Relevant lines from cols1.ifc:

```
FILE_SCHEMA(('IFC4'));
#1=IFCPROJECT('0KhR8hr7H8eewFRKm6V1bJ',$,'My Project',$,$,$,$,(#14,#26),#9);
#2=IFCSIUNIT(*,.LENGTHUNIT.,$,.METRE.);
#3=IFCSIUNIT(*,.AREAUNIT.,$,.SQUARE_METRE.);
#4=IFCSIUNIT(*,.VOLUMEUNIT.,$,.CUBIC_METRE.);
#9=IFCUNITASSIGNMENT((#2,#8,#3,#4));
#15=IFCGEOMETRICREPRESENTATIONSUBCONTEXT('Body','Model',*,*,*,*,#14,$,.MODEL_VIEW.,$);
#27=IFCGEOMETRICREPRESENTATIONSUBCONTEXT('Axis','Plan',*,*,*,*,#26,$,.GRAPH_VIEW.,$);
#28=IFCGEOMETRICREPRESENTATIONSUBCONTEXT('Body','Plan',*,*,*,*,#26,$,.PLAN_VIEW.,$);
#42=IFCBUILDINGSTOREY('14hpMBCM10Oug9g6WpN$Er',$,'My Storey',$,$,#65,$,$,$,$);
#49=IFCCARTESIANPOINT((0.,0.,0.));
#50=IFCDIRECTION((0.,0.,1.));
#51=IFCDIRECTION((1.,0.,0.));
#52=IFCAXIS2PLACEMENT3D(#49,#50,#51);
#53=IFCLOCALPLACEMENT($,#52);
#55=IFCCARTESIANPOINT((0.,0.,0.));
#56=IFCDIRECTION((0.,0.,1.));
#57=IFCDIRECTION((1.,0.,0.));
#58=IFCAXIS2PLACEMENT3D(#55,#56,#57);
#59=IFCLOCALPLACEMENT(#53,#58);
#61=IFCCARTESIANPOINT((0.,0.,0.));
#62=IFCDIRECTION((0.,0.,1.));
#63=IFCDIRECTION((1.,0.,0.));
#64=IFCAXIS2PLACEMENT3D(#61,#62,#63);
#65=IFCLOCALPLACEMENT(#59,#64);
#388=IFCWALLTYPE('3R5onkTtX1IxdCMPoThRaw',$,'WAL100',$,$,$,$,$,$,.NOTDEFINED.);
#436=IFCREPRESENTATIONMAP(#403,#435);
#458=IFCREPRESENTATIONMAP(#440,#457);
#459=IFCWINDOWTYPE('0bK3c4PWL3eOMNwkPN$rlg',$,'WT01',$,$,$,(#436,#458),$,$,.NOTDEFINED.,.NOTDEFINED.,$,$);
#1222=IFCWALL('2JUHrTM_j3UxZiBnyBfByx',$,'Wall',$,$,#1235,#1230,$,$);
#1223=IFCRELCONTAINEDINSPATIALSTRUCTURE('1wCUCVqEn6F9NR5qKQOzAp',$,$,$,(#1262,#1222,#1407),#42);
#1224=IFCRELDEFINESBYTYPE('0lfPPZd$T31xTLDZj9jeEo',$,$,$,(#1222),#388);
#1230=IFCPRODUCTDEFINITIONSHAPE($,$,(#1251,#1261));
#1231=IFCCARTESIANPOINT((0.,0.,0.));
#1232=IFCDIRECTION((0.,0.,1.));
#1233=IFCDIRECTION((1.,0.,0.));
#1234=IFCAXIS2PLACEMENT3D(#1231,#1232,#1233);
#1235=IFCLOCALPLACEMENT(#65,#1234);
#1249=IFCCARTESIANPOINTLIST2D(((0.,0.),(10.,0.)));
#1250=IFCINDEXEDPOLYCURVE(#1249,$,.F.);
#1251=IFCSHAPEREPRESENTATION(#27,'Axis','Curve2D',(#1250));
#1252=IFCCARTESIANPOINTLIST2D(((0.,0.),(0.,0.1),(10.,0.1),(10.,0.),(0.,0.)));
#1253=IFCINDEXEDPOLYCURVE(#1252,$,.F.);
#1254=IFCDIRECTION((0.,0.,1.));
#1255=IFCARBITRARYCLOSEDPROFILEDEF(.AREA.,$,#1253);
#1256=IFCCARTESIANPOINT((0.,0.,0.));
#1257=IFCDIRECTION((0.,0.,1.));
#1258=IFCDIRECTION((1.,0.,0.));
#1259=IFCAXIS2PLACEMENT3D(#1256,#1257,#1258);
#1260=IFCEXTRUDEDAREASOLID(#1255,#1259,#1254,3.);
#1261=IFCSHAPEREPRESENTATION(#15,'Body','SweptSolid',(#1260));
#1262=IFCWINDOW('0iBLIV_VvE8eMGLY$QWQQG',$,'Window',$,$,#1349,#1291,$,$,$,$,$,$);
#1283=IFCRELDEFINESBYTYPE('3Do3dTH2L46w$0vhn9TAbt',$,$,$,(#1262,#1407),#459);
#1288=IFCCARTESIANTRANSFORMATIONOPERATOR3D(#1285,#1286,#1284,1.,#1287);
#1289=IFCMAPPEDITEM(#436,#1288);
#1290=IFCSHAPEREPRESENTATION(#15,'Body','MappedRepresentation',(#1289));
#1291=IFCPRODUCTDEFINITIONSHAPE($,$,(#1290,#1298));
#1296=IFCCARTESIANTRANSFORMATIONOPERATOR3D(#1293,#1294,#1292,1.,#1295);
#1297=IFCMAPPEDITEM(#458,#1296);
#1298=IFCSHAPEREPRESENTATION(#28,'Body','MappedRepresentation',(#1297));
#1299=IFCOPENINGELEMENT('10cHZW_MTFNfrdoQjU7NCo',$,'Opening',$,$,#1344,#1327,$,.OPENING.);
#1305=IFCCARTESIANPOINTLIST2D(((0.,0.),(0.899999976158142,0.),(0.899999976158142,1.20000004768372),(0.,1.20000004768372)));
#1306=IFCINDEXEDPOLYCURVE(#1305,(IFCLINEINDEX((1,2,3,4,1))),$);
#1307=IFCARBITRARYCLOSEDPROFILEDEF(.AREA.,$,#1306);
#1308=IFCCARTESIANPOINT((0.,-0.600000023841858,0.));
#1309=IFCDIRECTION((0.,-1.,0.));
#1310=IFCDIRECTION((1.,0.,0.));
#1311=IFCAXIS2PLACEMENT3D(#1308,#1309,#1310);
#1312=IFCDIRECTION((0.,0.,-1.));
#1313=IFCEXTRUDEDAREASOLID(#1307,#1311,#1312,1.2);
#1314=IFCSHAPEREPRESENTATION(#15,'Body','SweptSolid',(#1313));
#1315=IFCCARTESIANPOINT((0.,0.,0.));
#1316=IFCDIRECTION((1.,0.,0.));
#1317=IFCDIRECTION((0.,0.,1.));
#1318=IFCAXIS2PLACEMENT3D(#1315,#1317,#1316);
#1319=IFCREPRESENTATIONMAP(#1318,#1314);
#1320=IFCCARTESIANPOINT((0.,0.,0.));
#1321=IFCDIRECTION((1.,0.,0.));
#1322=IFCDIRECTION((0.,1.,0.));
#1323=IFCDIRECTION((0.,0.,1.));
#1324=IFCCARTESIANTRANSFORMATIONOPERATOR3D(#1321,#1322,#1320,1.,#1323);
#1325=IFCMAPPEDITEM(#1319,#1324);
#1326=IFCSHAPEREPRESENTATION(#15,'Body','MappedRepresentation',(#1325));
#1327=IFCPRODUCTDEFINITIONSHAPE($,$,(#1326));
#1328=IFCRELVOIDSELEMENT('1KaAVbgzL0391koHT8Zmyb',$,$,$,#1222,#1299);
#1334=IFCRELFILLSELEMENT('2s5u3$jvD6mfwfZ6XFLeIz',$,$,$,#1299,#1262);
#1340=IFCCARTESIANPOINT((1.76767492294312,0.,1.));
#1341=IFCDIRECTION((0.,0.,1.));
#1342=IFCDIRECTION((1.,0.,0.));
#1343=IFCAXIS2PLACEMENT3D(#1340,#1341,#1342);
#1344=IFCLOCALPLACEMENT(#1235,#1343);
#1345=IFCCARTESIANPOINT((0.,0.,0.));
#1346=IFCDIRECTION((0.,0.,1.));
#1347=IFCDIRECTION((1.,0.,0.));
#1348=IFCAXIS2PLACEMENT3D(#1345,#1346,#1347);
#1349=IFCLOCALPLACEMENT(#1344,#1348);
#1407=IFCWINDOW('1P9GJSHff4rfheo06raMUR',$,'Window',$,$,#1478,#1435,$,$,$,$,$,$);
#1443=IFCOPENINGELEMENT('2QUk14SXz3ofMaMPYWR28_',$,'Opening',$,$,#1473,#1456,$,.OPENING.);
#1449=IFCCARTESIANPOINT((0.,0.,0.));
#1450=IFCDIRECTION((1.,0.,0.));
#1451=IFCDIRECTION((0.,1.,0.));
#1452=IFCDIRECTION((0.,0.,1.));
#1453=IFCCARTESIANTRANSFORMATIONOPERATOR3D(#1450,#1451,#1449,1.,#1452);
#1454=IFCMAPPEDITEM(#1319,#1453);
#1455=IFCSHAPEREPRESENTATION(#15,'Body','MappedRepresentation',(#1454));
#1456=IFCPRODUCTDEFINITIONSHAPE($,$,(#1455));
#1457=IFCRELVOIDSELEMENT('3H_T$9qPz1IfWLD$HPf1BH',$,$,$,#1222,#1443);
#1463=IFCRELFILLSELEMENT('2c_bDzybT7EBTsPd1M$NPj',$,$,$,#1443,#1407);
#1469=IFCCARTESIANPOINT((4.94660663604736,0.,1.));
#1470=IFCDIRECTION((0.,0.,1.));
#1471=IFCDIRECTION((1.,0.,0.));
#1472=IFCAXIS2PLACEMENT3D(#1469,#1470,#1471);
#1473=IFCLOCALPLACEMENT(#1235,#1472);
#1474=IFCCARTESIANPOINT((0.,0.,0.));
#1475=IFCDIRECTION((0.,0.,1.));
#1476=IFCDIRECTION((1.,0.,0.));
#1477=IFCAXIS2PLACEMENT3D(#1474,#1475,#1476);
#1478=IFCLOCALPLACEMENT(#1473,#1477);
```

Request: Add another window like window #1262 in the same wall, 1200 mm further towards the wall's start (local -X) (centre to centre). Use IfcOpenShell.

```python
import ifcopenshell
import ifcopenshell.api.feature
import ifcopenshell.api.geometry
import ifcopenshell.api.root
import ifcopenshell.geom
import ifcopenshell.util.element
import ifcopenshell.util.placement
import ifcopenshell.util.shape
import ifcopenshell.util.unit

model = ifcopenshell.open("cols1.ifc")
unit_scale = ifcopenshell.util.unit.calculate_unit_scale(model)
settings = ifcopenshell.geom.settings()


def volume(element):
    """Net volume in cubic metres, openings subtracted."""
    shape = ifcopenshell.geom.create_shape(settings, element)
    return ifcopenshell.util.shape.get_volume(shape.geometry)


window = model.by_id(1262)
opening = window.FillsVoids[0].RelatingOpeningElement
wall = opening.VoidsElements[0].RelatingBuildingElement
before = volume(wall)
shift = ifcopenshell.util.placement.get_local_placement(wall.ObjectPlacement)[:3, 0] * -1.2 / unit_scale

# copy_class copies the void relationship, type, container and properties, but no geometry.
new_opening = ifcopenshell.api.root.copy_class(model, product=opening)
new_opening.Representation = ifcopenshell.util.element.copy_deep(
    model, opening.Representation, exclude=["IfcGeometricRepresentationContext", "IfcRepresentationMap"]
)
new_window = ifcopenshell.api.root.copy_class(model, product=window)
new_window.Representation = ifcopenshell.util.element.copy_deep(
    model, window.Representation, exclude=["IfcGeometricRepresentationContext", "IfcRepresentationMap"]
)
ifcopenshell.api.feature.add_filling(model, opening=new_opening, element=new_window)

for old, new in ((opening, new_opening), (window, new_window)):
    matrix = ifcopenshell.util.placement.get_local_placement(old.ObjectPlacement)
    matrix[:3, 3] += shift
    ifcopenshell.api.geometry.edit_object_placement(model, product=new, matrix=matrix, is_si=False)

after = volume(wall)

print(f"wall volume {before:.3f} -> {after:.3f} m3")

model.write("cols1_updated.ifc")
```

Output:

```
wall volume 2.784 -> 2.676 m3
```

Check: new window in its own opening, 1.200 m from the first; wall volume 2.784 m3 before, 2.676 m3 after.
